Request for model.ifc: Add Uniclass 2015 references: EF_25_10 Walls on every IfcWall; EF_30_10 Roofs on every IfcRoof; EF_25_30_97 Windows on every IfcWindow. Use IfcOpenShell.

First a look at what the model holds.

```python
import ifcopenshell

model = ifcopenshell.open("model.ifc")
print(model.schema)
print("classifications:", [c.Name for c in model.by_type("IfcClassification")])
for ifc_class in ("IfcDoor", "IfcRoof", "IfcStair", "IfcWall", "IfcWindow"):
    print(ifc_class, len(model.by_type(ifc_class)))
```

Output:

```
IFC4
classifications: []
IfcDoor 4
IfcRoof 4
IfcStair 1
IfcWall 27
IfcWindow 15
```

```python
import ifcopenshell
import ifcopenshell.api.classification

model = ifcopenshell.open("model.ifc")

system = ifcopenshell.api.classification.add_classification(model, classification="Uniclass 2015")

codes = {
    "IfcWall": ("EF_25_10", "Walls"),
    "IfcRoof": ("EF_30_10", "Roofs"),
    "IfcWindow": ("EF_25_30_97", "Windows"),
}
for ifc_class, (code, name) in codes.items():
    products = model.by_type(ifc_class)
    ifcopenshell.api.classification.add_reference(
        model, products=products, classification=system, identification=code, name=name
    )
    print(code, len(products))

model.write("model_rev.ifc")
```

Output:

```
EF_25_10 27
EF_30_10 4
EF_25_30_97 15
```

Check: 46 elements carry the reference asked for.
